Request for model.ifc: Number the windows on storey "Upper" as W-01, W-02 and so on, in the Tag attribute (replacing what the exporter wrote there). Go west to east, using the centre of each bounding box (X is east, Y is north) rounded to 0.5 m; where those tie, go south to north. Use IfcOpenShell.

First a look at what the model holds.

```python
import ifcopenshell
import ifcopenshell.util.element
import ifcopenshell.util.placement

model = ifcopenshell.open("model.ifc")
print(model.schema)
storey = next(s for s in model.by_type("IfcBuildingStorey") if s.Name == "Upper")
windows = [e for e in ifcopenshell.util.element.get_decomposition(storey) if e.is_a("IfcWindow")]
for e in sorted(windows, key=lambda e: e.id()):
    origin = ifcopenshell.util.placement.get_local_placement(e.ObjectPlacement)[:3, 3]
    print(e.id(), e.Tag, e.Name, origin.round(2) + 0.0, sep=" | ")
```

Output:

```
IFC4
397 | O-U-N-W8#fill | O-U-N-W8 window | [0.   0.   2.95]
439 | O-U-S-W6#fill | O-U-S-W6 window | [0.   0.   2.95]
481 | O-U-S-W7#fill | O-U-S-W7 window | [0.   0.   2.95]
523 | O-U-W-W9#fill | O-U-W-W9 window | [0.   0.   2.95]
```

```python
import ifcopenshell
import ifcopenshell.geom
import ifcopenshell.util.element
import ifcopenshell.util.shape

model = ifcopenshell.open("model.ifc")
settings = ifcopenshell.geom.settings()
settings.set("use-world-coords", True)


def centre(element):
    shape = ifcopenshell.geom.create_shape(settings, element)
    return ifcopenshell.util.shape.get_bbox_centroid(shape.geometry)


storey = next(s for s in model.by_type("IfcBuildingStorey") if s.Name == "Upper")
windows = [e for e in ifcopenshell.util.element.get_decomposition(storey) if e.is_a("IfcWindow")]

# Insertion points can sit at a corner or the storey origin, so sort by the geometry (in metres).
centres = {e: centre(e) for e in windows}
windows.sort(key=lambda e: (round(centres[e][0] / 0.5), centres[e][1]))

for i, e in enumerate(windows, start=1):
    number = f"W-{i:02d}"
    e.Tag = number
    print(e.id(), number)

model.write("model_rev.ifc")
```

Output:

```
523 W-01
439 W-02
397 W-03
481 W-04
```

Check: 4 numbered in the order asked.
